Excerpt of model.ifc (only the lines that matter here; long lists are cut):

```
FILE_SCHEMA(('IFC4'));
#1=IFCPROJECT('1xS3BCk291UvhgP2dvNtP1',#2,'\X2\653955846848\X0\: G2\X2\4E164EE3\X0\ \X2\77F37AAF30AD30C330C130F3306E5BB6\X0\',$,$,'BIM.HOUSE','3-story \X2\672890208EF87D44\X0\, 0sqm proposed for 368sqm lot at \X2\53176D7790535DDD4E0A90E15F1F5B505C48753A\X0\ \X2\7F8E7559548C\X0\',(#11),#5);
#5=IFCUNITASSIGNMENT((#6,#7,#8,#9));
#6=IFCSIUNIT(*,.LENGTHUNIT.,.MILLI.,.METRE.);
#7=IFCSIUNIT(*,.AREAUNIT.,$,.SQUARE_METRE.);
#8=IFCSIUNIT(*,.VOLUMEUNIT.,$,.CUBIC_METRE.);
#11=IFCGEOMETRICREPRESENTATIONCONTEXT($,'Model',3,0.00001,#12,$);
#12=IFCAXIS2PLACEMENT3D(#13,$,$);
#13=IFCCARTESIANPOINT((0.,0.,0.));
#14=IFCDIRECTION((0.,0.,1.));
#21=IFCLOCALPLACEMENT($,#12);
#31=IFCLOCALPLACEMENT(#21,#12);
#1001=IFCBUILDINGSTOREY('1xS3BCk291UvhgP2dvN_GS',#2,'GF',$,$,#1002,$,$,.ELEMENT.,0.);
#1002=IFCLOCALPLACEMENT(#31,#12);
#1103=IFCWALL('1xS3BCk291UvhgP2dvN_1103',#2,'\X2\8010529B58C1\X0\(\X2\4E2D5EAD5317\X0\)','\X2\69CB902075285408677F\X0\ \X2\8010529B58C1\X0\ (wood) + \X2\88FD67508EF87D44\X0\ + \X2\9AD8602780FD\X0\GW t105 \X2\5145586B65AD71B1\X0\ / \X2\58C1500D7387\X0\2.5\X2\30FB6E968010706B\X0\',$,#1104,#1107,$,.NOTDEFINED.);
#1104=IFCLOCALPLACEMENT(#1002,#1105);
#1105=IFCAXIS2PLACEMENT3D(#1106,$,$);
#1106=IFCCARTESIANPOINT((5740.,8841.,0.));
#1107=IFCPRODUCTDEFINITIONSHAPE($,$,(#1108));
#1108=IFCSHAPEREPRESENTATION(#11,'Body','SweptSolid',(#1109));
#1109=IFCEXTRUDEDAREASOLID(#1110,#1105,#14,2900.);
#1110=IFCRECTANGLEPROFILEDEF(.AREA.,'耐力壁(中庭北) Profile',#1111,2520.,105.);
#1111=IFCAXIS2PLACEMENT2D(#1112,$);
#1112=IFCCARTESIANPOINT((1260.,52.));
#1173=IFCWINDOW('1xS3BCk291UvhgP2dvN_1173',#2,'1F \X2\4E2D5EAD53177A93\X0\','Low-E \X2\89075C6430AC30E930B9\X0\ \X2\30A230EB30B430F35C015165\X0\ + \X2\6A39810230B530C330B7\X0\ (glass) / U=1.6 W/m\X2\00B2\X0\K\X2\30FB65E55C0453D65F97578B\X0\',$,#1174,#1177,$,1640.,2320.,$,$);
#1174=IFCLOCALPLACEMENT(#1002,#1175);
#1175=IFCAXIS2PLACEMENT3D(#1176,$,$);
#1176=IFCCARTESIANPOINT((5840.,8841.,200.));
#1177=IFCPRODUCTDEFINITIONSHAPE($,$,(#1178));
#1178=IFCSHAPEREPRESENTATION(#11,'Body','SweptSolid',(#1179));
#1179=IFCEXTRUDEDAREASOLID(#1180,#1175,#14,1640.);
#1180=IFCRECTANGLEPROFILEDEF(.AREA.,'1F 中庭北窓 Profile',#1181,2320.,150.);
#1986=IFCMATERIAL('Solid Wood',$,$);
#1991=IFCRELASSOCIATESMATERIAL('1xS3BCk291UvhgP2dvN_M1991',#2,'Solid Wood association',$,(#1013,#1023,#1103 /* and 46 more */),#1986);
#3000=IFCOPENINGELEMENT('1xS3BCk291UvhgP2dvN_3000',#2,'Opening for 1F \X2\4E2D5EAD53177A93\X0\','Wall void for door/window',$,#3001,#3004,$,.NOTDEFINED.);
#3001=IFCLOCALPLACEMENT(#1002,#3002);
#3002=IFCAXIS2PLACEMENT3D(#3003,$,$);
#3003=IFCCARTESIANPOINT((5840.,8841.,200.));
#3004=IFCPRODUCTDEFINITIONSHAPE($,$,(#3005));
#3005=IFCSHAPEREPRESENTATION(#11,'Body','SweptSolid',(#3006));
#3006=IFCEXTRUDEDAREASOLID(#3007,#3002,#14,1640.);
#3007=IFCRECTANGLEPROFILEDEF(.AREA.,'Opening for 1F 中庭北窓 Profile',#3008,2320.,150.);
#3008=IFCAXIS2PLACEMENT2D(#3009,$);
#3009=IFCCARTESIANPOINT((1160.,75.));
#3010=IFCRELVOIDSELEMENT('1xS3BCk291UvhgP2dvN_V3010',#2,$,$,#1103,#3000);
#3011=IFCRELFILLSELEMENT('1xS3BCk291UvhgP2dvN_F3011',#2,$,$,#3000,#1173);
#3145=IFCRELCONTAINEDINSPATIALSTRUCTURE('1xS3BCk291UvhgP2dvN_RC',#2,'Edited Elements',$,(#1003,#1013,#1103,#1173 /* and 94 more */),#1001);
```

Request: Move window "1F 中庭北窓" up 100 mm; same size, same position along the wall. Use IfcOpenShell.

```python
import numpy as np
import ifcopenshell
import ifcopenshell.api.geometry
import ifcopenshell.util.placement
import ifcopenshell.util.unit

model = ifcopenshell.open("model.ifc")
unit_scale = ifcopenshell.util.unit.calculate_unit_scale(model)

window = model.by_guid("1xS3BCk291UvhgP2dvN_1173")
opening = window.FillsVoids[0].RelatingOpeningElement
dz = 0.1 / unit_scale

shift = np.array([0.0, 0.0, dz])
# The window is not placed relative to its opening, so move both.
for product in (opening, window):
    matrix = ifcopenshell.util.placement.get_local_placement(product.ObjectPlacement)
    matrix[:3, 3] += shift
    ifcopenshell.api.geometry.edit_object_placement(model, product=product, matrix=matrix, is_si=False)

print(f"moved by {dz * unit_scale:+.3f} m")

model.write("model_updated.ifc")
```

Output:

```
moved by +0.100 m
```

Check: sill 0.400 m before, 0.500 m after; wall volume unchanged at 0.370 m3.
